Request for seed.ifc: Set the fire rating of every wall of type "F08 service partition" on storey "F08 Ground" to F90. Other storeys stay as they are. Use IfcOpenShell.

First a look at what the model holds.

```python
import ifcopenshell
import ifcopenshell.util.element

model = ifcopenshell.open("seed.ifc")
print(model.schema)
storey = next(s for s in model.by_type("IfcBuildingStorey") if s.Name == "F08 Ground")
walls = [e for e in ifcopenshell.util.element.get_decomposition(storey) if e.is_a("IfcWall")]
seen = {}
for e in walls:
    element_type = ifcopenshell.util.element.get_type(e)
    key = (element_type.Name if element_type != e and element_type else None, ifcopenshell.util.element.get_pset(e, "Pset_WallCommon", "FireRating"))
    seen[key] = seen.get(key, 0) + 1
for (name, value), count in sorted(seen.items(), key=str):
    print(count, "x", name, "|", value)
```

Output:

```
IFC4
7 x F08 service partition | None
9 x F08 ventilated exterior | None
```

```python
import ifcopenshell
import ifcopenshell.api.pset
import ifcopenshell.util.element

model = ifcopenshell.open("seed.ifc")

storey = next(s for s in model.by_type("IfcBuildingStorey") if s.Name == "F08 Ground")
walls = [e for e in ifcopenshell.util.element.get_decomposition(storey) if e.is_a("IfcWall")]

count = 0
for e in walls:
    element_type = ifcopenshell.util.element.get_type(e)
    if element_type in (None, e) or element_type.Name != "F08 service partition":
        continue
    # add_pset returns the element's existing set when there is one.
    pset = ifcopenshell.api.pset.add_pset(model, product=e, name="Pset_WallCommon")
    ifcopenshell.api.pset.edit_pset(model, pset=pset, properties={"FireRating": "F90"})
    count += 1

print(count, "walls updated")

model.write("seed_updated.ifc")
```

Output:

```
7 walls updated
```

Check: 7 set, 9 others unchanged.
